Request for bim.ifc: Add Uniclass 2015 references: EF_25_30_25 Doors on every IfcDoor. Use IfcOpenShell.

First a look at what the model holds.

```python
import ifcopenshell

model = ifcopenshell.open("bim.ifc")
print(model.schema)
print("classifications:", [c.Name for c in model.by_type("IfcClassification")])
for ifc_class in ("IfcDoor", "IfcRoof", "IfcStair", "IfcWall", "IfcWindow"):
    print(ifc_class, len(model.by_type(ifc_class)))
```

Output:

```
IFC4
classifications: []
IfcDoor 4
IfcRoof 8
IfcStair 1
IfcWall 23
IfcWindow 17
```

```python
import ifcopenshell
import ifcopenshell.api.classification

model = ifcopenshell.open("bim.ifc")

system = ifcopenshell.api.classification.add_classification(model, classification="Uniclass 2015")

codes = {
    "IfcDoor": ("EF_25_30_25", "Doors"),
}
for ifc_class, (code, name) in codes.items():
    products = model.by_type(ifc_class)
    ifcopenshell.api.classification.add_reference(
        model, products=products, classification=system, identification=code, name=name
    )
    print(code, len(products))

model.write("bim_edited.ifc")
```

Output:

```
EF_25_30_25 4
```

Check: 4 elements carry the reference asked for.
